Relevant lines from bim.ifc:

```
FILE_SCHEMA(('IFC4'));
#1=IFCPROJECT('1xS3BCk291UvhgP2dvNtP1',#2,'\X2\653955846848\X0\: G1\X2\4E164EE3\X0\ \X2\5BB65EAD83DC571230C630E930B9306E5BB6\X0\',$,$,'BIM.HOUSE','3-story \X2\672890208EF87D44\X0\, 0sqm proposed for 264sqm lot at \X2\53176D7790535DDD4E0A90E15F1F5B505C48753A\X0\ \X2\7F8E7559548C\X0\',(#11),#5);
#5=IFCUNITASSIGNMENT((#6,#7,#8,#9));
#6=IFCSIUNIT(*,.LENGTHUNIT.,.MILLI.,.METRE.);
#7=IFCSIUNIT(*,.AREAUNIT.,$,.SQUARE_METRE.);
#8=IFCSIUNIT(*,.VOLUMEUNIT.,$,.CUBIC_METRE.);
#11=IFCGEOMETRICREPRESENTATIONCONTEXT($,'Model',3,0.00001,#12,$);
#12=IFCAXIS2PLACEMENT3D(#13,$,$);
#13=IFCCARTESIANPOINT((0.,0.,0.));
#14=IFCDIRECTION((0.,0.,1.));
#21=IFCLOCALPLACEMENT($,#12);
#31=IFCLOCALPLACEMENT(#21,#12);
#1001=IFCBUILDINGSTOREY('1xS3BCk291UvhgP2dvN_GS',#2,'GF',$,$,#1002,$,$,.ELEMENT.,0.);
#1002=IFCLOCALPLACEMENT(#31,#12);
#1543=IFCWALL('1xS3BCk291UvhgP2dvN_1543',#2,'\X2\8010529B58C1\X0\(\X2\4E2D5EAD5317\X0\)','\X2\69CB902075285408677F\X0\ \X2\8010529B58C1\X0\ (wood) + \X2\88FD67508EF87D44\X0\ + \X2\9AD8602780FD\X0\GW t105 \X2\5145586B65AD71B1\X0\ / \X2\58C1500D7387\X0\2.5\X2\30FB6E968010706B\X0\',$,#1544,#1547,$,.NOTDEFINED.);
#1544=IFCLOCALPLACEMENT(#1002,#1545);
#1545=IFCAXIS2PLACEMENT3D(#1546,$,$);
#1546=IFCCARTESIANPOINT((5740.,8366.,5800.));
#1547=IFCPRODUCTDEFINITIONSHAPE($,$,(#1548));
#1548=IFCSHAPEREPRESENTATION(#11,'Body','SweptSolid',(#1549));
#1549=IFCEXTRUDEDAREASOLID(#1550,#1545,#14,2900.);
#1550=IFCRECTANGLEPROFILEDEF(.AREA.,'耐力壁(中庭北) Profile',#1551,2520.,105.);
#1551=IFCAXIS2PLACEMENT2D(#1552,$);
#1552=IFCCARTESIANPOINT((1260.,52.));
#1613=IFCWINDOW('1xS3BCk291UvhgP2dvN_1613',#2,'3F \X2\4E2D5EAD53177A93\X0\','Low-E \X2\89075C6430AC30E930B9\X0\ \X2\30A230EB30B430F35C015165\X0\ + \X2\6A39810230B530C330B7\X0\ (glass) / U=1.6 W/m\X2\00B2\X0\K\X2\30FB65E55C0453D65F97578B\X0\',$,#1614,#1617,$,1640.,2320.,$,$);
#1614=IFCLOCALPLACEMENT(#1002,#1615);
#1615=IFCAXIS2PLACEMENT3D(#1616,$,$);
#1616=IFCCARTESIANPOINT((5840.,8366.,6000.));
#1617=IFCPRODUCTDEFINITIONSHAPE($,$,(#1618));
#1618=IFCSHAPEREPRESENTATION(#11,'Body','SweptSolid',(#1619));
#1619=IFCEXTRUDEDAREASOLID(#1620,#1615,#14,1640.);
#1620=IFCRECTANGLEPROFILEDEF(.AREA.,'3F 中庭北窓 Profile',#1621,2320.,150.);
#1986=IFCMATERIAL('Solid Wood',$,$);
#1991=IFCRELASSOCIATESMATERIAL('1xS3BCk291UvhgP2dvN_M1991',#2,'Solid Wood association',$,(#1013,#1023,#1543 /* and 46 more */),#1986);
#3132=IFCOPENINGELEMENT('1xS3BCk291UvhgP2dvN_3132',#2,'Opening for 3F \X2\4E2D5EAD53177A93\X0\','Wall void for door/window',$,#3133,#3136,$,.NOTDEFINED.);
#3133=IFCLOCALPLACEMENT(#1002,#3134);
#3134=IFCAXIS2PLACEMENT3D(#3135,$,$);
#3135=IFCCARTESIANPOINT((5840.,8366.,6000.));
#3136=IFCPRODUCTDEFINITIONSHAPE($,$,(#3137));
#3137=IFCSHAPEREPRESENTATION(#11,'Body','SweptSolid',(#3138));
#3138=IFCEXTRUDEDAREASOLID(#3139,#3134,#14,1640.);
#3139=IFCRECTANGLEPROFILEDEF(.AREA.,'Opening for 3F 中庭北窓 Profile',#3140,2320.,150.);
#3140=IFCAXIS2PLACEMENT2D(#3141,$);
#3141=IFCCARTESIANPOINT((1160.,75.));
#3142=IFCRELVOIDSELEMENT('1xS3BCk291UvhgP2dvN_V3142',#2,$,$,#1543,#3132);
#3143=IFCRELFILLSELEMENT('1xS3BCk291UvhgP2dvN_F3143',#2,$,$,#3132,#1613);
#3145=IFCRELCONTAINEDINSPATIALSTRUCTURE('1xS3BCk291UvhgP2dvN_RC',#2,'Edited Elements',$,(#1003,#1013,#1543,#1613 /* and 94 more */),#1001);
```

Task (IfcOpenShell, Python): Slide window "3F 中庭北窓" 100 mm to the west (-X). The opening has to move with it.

```python
import ifcopenshell
import ifcopenshell.api.geometry
import ifcopenshell.util.placement

model = ifcopenshell.open("bim.ifc")

window = model.by_id(1613)
opening = window.FillsVoids[0].RelatingOpeningElement
wall = opening.VoidsElements[0].RelatingBuildingElement

wall_matrix = ifcopenshell.util.placement.get_local_placement(wall.ObjectPlacement)
shift = wall_matrix[:3, 0] * -100.0
before = ifcopenshell.util.placement.get_local_placement(window.ObjectPlacement)[:3, 3].copy()

# The window is not placed relative to its opening, so move both.
for product in (opening, window):
    matrix = ifcopenshell.util.placement.get_local_placement(product.ObjectPlacement)
    matrix[:3, 3] += shift
    ifcopenshell.api.geometry.edit_object_placement(model, product=product, matrix=matrix, is_si=False)

after = ifcopenshell.util.placement.get_local_placement(window.ObjectPlacement)[:3, 3]
print("window moved by", (after - before).round(3) + 0.0)

model.write("bim_rev.ifc")
```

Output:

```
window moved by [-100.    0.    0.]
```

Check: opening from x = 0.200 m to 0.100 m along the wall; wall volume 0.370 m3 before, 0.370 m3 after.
